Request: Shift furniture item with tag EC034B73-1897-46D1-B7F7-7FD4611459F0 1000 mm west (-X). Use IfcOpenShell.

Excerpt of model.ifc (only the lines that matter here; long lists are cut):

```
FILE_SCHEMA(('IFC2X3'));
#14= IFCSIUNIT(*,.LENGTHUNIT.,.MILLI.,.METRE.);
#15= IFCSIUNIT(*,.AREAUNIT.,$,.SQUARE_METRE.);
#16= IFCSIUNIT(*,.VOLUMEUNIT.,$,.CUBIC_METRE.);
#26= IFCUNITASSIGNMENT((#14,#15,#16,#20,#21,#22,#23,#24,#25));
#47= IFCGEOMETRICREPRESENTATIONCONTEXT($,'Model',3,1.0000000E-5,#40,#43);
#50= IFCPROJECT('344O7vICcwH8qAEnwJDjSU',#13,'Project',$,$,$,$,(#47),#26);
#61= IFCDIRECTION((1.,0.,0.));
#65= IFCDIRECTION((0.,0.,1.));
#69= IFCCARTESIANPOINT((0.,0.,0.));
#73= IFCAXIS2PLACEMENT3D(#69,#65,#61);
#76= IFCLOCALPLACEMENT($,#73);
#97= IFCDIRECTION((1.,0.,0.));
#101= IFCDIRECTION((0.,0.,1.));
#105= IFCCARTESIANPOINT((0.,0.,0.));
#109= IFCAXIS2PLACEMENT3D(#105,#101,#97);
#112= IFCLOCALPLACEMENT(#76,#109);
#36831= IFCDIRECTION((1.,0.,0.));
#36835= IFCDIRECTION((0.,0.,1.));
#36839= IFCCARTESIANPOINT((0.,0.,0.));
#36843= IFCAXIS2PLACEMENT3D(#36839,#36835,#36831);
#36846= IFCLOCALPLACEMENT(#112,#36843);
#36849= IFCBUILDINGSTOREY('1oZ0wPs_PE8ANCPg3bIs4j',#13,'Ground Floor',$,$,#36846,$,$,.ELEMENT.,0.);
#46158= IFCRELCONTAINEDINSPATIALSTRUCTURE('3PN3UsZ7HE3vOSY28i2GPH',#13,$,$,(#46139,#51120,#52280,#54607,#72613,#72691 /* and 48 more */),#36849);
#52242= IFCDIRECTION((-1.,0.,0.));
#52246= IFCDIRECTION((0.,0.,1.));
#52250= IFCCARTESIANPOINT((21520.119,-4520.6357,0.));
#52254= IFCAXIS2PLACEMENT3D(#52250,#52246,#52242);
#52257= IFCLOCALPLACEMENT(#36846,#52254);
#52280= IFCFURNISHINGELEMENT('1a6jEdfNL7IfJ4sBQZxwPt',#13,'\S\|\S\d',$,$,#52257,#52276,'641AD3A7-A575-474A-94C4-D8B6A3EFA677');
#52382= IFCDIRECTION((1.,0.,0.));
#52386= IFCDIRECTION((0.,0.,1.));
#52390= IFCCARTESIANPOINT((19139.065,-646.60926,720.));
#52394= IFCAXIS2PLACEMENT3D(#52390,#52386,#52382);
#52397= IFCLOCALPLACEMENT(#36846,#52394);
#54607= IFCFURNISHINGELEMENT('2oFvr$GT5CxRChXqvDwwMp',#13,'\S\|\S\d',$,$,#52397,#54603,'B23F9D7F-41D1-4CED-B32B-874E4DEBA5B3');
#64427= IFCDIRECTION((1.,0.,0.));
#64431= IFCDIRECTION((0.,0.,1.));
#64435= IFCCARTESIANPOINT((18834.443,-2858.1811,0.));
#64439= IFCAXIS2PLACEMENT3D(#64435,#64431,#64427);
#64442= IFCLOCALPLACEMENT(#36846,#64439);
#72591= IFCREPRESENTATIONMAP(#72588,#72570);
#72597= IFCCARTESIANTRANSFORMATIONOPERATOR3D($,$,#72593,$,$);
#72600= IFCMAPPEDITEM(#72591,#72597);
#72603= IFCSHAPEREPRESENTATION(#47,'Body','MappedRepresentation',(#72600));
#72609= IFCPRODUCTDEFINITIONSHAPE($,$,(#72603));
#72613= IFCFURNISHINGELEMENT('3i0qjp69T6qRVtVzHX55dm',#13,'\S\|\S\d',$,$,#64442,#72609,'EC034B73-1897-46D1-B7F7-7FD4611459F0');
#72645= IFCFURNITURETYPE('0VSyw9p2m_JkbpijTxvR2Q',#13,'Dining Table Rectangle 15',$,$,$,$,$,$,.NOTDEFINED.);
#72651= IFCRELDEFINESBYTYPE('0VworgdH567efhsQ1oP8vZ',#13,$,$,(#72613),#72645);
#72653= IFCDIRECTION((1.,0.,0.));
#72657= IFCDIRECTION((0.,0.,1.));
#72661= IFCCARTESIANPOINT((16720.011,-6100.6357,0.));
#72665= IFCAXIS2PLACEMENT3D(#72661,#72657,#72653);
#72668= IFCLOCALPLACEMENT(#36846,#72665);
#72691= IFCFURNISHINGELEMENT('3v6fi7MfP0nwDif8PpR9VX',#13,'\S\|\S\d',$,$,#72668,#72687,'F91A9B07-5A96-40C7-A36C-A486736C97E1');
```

```python
import ifcopenshell
import ifcopenshell.api.geometry
import ifcopenshell.util.placement
import ifcopenshell.util.unit

model = ifcopenshell.open("model.ifc")
unit_scale = ifcopenshell.util.unit.calculate_unit_scale(model)

item = model.by_guid("3i0qjp69T6qRVtVzHX55dm")
matrix = ifcopenshell.util.placement.get_local_placement(item.ObjectPlacement)
matrix[0, 3] -= 1 / unit_scale
ifcopenshell.api.geometry.edit_object_placement(model, product=item, matrix=matrix, is_si=False)

print(ifcopenshell.util.placement.get_local_placement(item.ObjectPlacement).round(3) + 0.0)

model.write("model_rev.ifc")
```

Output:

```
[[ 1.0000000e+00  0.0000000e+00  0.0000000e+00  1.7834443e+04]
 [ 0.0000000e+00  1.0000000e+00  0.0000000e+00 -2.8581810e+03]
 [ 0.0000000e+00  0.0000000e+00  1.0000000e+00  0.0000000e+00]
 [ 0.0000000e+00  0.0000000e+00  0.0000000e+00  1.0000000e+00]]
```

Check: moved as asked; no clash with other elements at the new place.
